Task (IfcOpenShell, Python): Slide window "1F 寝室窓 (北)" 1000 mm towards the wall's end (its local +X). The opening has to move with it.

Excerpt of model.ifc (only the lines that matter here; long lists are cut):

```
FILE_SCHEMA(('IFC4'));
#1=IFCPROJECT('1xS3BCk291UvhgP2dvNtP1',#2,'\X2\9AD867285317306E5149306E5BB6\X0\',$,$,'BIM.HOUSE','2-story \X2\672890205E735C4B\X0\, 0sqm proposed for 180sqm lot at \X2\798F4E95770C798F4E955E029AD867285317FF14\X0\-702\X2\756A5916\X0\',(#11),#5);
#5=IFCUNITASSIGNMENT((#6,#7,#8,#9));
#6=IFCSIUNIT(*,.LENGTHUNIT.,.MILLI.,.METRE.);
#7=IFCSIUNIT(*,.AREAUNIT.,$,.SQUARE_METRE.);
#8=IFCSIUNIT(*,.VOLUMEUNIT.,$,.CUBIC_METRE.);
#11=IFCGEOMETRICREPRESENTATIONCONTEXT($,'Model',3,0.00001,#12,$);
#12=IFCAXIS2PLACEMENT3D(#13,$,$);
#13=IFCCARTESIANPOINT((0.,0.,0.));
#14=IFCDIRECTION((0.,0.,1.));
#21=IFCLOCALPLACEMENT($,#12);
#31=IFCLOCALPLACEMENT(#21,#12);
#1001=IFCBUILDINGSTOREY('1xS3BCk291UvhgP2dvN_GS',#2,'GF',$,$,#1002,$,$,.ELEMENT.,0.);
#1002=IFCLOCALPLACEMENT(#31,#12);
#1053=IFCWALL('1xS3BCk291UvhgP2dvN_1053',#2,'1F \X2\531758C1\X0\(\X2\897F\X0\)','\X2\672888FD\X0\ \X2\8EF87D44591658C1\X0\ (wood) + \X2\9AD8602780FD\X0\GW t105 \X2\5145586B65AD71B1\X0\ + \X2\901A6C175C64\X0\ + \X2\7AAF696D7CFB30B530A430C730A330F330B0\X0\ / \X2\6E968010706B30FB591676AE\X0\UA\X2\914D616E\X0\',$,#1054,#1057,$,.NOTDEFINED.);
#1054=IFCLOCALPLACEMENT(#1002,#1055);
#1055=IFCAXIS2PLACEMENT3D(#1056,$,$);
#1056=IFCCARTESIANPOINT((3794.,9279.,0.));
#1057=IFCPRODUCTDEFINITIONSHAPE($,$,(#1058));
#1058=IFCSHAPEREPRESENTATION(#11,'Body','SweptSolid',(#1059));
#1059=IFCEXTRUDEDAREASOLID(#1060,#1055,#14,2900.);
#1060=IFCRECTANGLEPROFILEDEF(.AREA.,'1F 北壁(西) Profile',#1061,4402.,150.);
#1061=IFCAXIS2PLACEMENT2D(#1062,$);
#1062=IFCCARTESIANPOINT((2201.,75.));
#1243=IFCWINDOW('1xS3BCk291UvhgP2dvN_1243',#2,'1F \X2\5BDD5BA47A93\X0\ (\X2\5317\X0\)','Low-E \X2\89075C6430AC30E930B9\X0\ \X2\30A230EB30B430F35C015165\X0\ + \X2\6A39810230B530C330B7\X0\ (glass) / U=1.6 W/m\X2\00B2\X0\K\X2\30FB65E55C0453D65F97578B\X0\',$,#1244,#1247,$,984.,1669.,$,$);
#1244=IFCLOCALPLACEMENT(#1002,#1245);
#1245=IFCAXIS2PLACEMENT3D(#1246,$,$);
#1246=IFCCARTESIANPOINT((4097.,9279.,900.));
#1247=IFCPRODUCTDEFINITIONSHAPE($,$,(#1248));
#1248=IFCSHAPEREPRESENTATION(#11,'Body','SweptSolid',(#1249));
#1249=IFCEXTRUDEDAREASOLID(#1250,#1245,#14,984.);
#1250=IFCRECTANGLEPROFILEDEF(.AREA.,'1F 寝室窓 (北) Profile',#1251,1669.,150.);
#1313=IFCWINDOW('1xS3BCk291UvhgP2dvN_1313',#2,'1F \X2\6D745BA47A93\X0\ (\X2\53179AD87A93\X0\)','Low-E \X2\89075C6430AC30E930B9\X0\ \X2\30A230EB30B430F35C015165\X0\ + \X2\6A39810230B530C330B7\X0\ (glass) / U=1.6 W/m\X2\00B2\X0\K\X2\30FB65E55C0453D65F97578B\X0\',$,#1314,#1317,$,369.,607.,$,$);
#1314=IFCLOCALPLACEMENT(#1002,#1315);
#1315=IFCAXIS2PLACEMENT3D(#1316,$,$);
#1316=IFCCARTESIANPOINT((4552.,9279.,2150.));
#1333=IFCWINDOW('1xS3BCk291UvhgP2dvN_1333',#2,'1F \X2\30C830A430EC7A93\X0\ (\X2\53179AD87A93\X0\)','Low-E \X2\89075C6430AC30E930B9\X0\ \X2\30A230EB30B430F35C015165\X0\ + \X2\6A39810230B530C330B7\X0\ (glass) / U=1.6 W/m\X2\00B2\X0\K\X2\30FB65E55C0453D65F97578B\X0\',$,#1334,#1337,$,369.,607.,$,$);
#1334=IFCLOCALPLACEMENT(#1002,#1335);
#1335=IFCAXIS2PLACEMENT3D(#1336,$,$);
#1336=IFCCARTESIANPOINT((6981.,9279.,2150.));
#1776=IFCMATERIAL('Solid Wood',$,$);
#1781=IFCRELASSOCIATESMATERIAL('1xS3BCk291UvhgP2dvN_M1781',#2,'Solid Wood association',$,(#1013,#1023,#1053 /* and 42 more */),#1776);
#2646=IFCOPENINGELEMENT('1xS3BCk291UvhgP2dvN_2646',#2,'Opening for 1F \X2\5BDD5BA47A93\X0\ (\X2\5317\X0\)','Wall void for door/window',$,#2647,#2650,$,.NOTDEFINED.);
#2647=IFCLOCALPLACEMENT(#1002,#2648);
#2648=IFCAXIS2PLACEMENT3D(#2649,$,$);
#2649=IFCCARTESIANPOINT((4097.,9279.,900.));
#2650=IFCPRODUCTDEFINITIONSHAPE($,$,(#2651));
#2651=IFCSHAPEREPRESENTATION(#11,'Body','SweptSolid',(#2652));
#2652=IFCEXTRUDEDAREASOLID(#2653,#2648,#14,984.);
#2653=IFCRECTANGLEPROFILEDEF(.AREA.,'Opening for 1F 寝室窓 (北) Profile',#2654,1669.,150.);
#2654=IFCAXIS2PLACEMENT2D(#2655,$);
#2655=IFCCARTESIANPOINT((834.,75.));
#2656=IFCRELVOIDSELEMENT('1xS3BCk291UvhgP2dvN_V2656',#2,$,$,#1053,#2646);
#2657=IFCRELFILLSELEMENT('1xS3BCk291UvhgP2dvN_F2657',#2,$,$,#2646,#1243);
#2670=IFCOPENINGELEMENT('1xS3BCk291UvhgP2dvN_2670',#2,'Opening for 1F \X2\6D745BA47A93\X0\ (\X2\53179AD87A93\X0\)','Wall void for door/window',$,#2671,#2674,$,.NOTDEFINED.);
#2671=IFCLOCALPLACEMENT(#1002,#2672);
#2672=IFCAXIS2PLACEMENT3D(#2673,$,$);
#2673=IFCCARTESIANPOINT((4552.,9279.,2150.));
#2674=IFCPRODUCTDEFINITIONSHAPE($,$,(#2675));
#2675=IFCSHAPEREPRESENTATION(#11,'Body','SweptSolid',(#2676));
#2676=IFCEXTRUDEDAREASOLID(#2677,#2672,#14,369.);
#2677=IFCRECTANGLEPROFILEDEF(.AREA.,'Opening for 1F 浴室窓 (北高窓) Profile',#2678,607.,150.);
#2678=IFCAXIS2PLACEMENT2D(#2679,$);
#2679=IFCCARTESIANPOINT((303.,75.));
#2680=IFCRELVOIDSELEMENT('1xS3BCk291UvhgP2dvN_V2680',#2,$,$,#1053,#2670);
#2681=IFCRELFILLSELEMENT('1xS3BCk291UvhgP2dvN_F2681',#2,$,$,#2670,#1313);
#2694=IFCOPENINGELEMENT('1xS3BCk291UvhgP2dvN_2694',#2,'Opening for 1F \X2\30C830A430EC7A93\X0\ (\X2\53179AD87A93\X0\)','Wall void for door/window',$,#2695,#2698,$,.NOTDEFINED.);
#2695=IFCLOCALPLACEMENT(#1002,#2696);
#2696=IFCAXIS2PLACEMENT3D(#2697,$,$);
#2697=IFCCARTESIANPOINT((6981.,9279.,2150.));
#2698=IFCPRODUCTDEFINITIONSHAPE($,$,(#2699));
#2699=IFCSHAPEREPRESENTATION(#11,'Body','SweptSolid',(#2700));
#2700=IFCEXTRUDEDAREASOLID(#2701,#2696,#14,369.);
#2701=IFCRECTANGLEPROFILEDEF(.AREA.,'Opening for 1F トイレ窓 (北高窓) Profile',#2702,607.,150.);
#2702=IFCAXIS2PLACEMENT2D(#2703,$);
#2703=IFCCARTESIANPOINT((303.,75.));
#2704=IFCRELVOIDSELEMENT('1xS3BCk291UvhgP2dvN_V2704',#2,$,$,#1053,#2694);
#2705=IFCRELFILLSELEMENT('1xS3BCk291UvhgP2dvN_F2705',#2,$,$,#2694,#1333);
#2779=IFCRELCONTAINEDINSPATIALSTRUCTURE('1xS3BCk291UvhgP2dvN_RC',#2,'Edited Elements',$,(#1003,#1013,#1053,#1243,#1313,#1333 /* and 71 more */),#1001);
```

```python
import ifcopenshell
import ifcopenshell.api.geometry
import ifcopenshell.util.placement
import ifcopenshell.util.unit

model = ifcopenshell.open("model.ifc")
unit_scale = ifcopenshell.util.unit.calculate_unit_scale(model)

window = model.by_guid("1xS3BCk291UvhgP2dvN_1243")
opening = window.FillsVoids[0].RelatingOpeningElement
wall = opening.VoidsElements[0].RelatingBuildingElement

wall_matrix = ifcopenshell.util.placement.get_local_placement(wall.ObjectPlacement)
shift = wall_matrix[:3, 0] * 1 / unit_scale
before = ifcopenshell.util.placement.get_local_placement(window.ObjectPlacement)[:3, 3].copy()

# The window is not placed relative to its opening, so move both.
for product in (opening, window):
    matrix = ifcopenshell.util.placement.get_local_placement(product.ObjectPlacement)
    matrix[:3, 3] += shift
    ifcopenshell.api.geometry.edit_object_placement(model, product=product, matrix=matrix, is_si=False)

after = ifcopenshell.util.placement.get_local_placement(window.ObjectPlacement)[:3, 3]
print("window moved by", (after - before).round(3) + 0.0)

model.write("model-out.ifc")
```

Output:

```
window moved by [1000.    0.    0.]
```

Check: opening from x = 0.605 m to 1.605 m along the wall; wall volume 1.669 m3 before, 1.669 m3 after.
